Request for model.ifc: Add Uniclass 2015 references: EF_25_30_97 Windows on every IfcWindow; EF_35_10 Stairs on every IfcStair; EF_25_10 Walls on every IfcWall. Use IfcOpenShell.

First a look at what the model holds.

```python
import ifcopenshell

model = ifcopenshell.open("model.ifc")
print(model.schema)
print("classifications:", [c.Name for c in model.by_type("IfcClassification")])
for ifc_class in ("IfcDoor", "IfcRoof", "IfcStair", "IfcWall", "IfcWindow"):
    print(ifc_class, len(model.by_type(ifc_class)))
```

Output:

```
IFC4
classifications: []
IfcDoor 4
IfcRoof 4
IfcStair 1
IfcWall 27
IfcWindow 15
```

```python
import ifcopenshell
import ifcopenshell.api.classification

model = ifcopenshell.open("model.ifc")

system = ifcopenshell.api.classification.add_classification(model, classification="Uniclass 2015")

codes = {
    "IfcWindow": ("EF_25_30_97", "Windows"),
    "IfcStair": ("EF_35_10", "Stairs"),
    "IfcWall": ("EF_25_10", "Walls"),
}
for ifc_class, (code, name) in codes.items():
    products = model.by_type(ifc_class)
    ifcopenshell.api.classification.add_reference(
        model, products=products, classification=system, identification=code, name=name
    )
    print(code, len(products))

model.write("model_updated.ifc")
```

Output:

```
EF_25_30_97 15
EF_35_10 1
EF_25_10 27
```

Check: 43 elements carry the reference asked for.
